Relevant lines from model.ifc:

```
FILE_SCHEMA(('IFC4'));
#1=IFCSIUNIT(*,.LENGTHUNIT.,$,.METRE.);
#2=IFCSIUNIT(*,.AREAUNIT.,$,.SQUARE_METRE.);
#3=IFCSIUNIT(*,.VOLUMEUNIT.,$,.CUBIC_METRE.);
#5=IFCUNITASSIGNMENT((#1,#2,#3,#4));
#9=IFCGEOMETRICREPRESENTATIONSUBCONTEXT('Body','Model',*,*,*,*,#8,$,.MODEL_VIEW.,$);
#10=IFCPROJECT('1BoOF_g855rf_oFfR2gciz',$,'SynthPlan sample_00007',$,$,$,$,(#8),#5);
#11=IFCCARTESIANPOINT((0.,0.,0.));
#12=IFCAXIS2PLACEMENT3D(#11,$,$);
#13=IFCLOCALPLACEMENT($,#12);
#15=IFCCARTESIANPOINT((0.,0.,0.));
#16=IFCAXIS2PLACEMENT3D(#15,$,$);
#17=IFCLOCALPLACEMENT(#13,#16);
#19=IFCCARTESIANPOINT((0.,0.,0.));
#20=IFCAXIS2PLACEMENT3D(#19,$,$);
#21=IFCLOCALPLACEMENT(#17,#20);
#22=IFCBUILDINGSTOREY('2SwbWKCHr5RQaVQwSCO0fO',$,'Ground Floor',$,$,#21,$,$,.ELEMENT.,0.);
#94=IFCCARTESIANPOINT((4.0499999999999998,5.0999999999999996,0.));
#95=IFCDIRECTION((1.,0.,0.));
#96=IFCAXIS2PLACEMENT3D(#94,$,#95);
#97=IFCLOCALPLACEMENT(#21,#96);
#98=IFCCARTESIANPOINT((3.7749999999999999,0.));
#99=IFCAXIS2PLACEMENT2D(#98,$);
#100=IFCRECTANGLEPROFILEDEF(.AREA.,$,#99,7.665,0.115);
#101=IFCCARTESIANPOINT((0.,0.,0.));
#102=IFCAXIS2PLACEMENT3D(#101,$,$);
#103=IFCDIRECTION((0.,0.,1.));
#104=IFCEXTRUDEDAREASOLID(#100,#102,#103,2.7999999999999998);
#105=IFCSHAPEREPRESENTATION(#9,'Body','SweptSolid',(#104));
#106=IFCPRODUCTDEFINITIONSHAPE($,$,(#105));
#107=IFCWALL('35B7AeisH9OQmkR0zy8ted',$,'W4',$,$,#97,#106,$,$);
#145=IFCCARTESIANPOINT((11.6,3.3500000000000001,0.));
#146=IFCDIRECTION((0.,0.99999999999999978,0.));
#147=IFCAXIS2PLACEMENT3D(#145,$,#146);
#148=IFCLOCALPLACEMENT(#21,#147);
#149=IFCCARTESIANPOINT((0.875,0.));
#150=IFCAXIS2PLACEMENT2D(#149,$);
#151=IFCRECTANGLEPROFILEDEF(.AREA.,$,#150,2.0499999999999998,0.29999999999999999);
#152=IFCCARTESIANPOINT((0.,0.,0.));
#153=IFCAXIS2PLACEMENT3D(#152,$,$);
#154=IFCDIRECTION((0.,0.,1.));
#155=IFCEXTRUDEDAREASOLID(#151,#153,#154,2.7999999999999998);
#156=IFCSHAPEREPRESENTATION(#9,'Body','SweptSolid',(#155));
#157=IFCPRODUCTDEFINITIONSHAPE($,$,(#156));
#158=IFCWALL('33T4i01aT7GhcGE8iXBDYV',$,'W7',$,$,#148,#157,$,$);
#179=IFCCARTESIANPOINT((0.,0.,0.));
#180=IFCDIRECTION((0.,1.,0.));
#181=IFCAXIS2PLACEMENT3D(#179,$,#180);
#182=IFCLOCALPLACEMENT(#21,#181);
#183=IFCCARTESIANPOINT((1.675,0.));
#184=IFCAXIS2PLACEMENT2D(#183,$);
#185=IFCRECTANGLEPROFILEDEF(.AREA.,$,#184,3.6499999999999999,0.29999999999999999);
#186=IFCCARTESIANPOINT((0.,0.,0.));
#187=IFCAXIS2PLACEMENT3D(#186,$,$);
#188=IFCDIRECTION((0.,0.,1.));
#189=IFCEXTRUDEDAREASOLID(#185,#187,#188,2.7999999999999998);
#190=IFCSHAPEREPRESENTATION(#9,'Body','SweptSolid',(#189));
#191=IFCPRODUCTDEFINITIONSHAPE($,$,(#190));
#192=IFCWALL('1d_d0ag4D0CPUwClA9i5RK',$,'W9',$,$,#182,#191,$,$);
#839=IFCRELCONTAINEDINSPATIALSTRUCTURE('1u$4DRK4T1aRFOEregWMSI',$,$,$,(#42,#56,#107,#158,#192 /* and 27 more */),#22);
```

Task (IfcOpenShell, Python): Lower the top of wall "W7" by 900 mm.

```python
import ifcopenshell
import ifcopenshell.geom
import ifcopenshell.util.representation
import ifcopenshell.util.shape
import ifcopenshell.util.unit

model = ifcopenshell.open("model.ifc")
unit_scale = ifcopenshell.util.unit.calculate_unit_scale(model)
settings = ifcopenshell.geom.settings()


def volume(element):
    """Net volume in cubic metres, openings subtracted."""
    shape = ifcopenshell.geom.create_shape(settings, element)
    return ifcopenshell.util.shape.get_volume(shape.geometry)


wall = model.by_id(158)
before = volume(wall)

body = ifcopenshell.util.representation.get_representation(wall, "Model", "Body")
solid = body.Items[0]
old_height = solid.Depth
solid.Depth -= 0.9 / unit_scale
after = volume(wall)

print(f"height {old_height:g} -> {solid.Depth:g}, volume {before:.3f} -> {after:.3f} m3")

model.write("model_edited.ifc")
```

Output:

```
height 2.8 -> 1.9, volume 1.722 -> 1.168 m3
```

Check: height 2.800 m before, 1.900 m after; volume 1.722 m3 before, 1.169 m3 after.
